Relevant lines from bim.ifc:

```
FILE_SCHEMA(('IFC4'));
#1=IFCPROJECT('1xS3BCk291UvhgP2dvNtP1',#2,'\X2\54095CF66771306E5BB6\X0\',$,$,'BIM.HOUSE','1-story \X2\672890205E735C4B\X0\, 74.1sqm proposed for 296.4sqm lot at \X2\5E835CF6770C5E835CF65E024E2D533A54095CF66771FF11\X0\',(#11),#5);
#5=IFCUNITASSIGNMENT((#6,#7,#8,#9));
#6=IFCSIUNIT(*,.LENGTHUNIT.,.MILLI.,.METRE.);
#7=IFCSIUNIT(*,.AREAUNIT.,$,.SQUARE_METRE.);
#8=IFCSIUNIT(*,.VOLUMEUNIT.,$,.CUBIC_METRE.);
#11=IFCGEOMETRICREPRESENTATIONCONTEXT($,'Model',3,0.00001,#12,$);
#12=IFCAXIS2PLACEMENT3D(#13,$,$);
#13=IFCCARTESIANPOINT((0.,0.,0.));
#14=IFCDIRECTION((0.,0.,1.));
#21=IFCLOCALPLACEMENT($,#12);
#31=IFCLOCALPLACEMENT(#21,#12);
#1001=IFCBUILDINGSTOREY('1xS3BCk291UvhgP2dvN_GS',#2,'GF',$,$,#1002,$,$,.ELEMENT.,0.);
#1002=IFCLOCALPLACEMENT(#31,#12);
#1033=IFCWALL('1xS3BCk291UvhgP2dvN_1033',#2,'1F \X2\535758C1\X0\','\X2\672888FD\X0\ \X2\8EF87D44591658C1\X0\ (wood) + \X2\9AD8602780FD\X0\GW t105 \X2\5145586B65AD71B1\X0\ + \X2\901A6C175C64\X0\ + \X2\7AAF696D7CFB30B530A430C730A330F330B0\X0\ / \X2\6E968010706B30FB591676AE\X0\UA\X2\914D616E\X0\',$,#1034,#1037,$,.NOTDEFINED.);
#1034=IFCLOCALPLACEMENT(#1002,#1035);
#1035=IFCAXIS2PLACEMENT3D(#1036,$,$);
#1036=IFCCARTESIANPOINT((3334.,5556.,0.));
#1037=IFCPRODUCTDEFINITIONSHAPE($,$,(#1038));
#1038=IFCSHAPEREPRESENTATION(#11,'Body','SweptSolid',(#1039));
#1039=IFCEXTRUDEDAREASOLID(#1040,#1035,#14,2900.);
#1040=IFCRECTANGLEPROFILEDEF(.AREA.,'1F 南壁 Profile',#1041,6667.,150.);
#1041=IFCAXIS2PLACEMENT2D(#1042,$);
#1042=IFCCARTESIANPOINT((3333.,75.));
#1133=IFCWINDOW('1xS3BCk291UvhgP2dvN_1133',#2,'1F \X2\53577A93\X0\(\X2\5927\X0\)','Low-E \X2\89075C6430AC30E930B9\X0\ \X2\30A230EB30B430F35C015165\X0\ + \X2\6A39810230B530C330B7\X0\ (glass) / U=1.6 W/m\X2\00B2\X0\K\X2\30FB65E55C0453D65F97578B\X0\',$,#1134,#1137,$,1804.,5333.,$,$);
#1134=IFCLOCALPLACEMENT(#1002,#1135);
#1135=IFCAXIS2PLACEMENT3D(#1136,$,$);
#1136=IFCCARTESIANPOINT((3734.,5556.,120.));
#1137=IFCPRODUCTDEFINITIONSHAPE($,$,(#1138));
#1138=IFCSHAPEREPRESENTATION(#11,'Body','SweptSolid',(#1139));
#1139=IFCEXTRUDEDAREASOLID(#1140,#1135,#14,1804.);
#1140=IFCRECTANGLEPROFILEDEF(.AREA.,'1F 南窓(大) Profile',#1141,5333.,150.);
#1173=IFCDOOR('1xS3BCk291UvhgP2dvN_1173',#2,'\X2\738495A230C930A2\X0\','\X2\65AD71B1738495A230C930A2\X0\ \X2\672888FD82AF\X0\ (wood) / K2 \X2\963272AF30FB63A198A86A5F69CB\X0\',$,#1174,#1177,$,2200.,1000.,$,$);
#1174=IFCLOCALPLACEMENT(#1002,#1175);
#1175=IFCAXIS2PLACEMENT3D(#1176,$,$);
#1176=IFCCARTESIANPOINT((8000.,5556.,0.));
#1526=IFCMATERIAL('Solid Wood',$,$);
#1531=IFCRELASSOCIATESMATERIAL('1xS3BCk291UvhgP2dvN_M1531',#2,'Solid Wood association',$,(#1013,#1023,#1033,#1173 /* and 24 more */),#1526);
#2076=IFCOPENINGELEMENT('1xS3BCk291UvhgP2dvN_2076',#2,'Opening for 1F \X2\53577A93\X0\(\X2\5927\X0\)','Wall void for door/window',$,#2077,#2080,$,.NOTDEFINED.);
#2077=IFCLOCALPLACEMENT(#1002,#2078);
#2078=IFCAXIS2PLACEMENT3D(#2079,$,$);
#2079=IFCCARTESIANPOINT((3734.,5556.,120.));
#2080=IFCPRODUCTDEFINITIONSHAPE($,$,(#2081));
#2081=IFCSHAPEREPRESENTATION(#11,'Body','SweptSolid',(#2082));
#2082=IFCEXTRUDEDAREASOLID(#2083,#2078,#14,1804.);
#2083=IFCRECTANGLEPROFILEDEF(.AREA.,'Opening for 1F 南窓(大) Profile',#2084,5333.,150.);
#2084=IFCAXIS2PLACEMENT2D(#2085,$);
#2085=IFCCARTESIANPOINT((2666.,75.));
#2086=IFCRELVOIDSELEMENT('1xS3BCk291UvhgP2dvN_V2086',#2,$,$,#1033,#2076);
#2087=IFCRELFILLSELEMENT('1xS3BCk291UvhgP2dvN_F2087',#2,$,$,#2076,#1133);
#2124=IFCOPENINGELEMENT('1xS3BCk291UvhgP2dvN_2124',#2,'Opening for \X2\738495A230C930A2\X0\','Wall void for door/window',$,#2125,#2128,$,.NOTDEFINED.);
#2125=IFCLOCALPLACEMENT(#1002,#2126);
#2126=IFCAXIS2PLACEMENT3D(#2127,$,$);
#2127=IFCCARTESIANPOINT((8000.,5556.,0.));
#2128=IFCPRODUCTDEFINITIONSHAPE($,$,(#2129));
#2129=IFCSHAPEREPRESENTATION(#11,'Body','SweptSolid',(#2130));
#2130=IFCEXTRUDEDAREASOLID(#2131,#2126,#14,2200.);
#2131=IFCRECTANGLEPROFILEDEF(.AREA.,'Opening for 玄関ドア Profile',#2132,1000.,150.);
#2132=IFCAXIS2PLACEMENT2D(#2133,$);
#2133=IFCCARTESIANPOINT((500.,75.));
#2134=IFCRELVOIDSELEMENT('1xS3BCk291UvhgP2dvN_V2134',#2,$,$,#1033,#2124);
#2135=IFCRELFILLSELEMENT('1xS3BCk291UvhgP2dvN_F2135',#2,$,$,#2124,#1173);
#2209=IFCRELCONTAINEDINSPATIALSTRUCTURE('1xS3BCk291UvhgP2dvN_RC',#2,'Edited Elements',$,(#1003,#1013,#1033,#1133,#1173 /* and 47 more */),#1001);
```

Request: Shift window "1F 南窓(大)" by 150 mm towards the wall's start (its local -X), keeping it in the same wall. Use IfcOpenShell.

```python
import ifcopenshell
import ifcopenshell.api.geometry
import ifcopenshell.util.placement

model = ifcopenshell.open("bim.ifc")

window = model.by_guid("1xS3BCk291UvhgP2dvN_1133")
opening = window.FillsVoids[0].RelatingOpeningElement
wall = opening.VoidsElements[0].RelatingBuildingElement

wall_matrix = ifcopenshell.util.placement.get_local_placement(wall.ObjectPlacement)
shift = wall_matrix[:3, 0] * -150.0
before = ifcopenshell.util.placement.get_local_placement(window.ObjectPlacement)[:3, 3].copy()

# The window is not placed relative to its opening, so move both.
for product in (opening, window):
    matrix = ifcopenshell.util.placement.get_local_placement(product.ObjectPlacement)
    matrix[:3, 3] += shift
    ifcopenshell.api.geometry.edit_object_placement(model, product=product, matrix=matrix, is_si=False)

after = ifcopenshell.util.placement.get_local_placement(window.ObjectPlacement)[:3, 3]
print("window moved by", (after - before).round(3) + 0.0)

model.write("bim_v2.ifc")
```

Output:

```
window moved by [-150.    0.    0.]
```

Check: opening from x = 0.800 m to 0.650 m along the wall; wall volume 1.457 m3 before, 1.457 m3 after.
